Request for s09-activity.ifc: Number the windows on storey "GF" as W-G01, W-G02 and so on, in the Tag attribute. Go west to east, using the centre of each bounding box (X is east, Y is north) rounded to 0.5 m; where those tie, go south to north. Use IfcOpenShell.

First a look at what the model holds.

```python
import ifcopenshell
import ifcopenshell.util.element
import ifcopenshell.util.placement

model = ifcopenshell.open("s09-activity.ifc")
print(model.schema)
storey = next(s for s in model.by_type("IfcBuildingStorey") if s.Name == "GF")
windows = [e for e in ifcopenshell.util.element.get_decomposition(storey) if e.is_a("IfcWindow")]
for e in sorted(windows, key=lambda e: e.id()):
    origin = ifcopenshell.util.placement.get_local_placement(e.ObjectPlacement)[:3, 3]
    print(e.id(), e.Tag, e.Name, origin.round(2) + 0.0, sep=" | ")
```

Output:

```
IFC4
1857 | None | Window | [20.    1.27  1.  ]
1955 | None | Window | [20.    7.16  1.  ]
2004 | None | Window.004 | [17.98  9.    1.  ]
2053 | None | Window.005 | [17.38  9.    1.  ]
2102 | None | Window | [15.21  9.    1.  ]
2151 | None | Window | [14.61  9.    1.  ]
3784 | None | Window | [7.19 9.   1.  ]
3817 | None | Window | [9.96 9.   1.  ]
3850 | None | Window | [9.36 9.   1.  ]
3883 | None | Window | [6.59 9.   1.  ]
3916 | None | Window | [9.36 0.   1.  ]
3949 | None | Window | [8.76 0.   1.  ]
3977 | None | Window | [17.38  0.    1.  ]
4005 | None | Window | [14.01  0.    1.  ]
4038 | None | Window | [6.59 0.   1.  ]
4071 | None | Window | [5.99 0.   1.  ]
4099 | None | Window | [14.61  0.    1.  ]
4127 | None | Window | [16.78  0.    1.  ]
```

```python
import ifcopenshell
import ifcopenshell.geom
import ifcopenshell.util.element
import ifcopenshell.util.shape

model = ifcopenshell.open("s09-activity.ifc")
settings = ifcopenshell.geom.settings()
settings.set("use-world-coords", True)


def centre(element):
    shape = ifcopenshell.geom.create_shape(settings, element)
    return ifcopenshell.util.shape.get_bbox_centroid(shape.geometry)


storey = next(s for s in model.by_type("IfcBuildingStorey") if s.Name == "GF")
windows = [e for e in ifcopenshell.util.element.get_decomposition(storey) if e.is_a("IfcWindow")]

# Insertion points can sit at a corner or the storey origin, so sort by the geometry (in metres).
centres = {e: centre(e) for e in windows}
windows.sort(key=lambda e: (round(centres[e][0] / 0.5), centres[e][1]))

for i, e in enumerate(windows, start=1):
    number = f"W-G{i:02d}"
    e.Tag = number
    print(e.id(), number)

model.write("s09-activity_v2.ifc")
```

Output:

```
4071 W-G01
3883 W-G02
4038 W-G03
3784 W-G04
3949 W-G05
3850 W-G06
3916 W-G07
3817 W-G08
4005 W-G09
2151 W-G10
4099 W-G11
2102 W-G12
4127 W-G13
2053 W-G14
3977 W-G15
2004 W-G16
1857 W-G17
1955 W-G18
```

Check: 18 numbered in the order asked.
